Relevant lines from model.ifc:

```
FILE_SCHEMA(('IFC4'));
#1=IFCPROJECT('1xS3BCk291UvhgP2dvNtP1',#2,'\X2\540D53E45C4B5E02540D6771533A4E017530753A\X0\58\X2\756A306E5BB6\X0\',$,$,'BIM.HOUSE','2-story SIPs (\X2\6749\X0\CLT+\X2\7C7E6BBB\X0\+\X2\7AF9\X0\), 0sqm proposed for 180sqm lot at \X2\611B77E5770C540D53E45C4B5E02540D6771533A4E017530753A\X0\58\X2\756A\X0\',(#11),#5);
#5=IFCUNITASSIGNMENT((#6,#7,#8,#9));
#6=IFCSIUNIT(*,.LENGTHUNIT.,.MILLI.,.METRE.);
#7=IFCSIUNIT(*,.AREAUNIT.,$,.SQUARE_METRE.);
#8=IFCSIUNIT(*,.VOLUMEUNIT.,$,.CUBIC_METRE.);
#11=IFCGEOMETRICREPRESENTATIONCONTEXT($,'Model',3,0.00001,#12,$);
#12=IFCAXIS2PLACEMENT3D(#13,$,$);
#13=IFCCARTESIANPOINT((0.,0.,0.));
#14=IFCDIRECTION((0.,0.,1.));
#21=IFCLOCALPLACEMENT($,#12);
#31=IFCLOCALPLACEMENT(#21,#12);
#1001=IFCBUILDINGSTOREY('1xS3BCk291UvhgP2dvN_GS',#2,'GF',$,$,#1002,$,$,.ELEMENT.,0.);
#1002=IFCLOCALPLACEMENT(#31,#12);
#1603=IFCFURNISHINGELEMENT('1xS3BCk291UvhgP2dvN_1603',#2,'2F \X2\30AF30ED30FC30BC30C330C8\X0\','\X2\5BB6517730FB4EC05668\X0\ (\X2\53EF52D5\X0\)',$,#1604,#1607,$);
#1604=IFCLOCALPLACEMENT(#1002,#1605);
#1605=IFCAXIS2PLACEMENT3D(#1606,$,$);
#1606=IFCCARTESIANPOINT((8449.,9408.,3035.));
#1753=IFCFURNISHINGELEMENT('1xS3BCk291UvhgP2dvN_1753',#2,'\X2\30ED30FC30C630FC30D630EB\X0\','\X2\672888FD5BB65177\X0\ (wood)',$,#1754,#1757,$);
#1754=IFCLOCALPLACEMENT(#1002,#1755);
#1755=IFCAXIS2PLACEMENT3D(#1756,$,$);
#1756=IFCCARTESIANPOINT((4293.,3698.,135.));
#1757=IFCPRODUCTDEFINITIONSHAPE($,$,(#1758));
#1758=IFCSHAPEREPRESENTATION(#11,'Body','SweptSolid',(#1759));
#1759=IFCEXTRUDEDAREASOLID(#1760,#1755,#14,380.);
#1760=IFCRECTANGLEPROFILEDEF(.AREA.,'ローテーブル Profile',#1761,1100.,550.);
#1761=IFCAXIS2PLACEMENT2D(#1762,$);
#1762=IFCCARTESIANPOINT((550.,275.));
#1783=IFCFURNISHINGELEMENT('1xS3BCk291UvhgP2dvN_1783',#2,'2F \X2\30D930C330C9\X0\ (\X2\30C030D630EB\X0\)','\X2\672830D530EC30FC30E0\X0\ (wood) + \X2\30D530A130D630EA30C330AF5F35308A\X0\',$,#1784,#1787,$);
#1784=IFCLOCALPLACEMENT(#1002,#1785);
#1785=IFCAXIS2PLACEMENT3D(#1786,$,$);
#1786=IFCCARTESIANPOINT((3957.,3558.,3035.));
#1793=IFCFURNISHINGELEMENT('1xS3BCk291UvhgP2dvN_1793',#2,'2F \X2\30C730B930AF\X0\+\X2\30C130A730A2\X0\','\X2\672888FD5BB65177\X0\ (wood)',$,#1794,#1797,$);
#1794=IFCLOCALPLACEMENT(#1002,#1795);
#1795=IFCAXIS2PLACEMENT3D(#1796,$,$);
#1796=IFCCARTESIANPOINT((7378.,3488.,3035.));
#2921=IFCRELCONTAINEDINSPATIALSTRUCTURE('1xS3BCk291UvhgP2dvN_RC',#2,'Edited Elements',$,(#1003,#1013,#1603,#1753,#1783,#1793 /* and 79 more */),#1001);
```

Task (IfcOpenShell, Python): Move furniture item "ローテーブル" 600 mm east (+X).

```python
import ifcopenshell
import ifcopenshell.api.geometry
import ifcopenshell.util.placement

model = ifcopenshell.open("model.ifc")

item = model.by_guid("1xS3BCk291UvhgP2dvN_1753")
matrix = ifcopenshell.util.placement.get_local_placement(item.ObjectPlacement)
matrix[0, 3] += 600.0
ifcopenshell.api.geometry.edit_object_placement(model, product=item, matrix=matrix, is_si=False)

print(ifcopenshell.util.placement.get_local_placement(item.ObjectPlacement).round(3) + 0.0)

model.write("model_edited.ifc")
```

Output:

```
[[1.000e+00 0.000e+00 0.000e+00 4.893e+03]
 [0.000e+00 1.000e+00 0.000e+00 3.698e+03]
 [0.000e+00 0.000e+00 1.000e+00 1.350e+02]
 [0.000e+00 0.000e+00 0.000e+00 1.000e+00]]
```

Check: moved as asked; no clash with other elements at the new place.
